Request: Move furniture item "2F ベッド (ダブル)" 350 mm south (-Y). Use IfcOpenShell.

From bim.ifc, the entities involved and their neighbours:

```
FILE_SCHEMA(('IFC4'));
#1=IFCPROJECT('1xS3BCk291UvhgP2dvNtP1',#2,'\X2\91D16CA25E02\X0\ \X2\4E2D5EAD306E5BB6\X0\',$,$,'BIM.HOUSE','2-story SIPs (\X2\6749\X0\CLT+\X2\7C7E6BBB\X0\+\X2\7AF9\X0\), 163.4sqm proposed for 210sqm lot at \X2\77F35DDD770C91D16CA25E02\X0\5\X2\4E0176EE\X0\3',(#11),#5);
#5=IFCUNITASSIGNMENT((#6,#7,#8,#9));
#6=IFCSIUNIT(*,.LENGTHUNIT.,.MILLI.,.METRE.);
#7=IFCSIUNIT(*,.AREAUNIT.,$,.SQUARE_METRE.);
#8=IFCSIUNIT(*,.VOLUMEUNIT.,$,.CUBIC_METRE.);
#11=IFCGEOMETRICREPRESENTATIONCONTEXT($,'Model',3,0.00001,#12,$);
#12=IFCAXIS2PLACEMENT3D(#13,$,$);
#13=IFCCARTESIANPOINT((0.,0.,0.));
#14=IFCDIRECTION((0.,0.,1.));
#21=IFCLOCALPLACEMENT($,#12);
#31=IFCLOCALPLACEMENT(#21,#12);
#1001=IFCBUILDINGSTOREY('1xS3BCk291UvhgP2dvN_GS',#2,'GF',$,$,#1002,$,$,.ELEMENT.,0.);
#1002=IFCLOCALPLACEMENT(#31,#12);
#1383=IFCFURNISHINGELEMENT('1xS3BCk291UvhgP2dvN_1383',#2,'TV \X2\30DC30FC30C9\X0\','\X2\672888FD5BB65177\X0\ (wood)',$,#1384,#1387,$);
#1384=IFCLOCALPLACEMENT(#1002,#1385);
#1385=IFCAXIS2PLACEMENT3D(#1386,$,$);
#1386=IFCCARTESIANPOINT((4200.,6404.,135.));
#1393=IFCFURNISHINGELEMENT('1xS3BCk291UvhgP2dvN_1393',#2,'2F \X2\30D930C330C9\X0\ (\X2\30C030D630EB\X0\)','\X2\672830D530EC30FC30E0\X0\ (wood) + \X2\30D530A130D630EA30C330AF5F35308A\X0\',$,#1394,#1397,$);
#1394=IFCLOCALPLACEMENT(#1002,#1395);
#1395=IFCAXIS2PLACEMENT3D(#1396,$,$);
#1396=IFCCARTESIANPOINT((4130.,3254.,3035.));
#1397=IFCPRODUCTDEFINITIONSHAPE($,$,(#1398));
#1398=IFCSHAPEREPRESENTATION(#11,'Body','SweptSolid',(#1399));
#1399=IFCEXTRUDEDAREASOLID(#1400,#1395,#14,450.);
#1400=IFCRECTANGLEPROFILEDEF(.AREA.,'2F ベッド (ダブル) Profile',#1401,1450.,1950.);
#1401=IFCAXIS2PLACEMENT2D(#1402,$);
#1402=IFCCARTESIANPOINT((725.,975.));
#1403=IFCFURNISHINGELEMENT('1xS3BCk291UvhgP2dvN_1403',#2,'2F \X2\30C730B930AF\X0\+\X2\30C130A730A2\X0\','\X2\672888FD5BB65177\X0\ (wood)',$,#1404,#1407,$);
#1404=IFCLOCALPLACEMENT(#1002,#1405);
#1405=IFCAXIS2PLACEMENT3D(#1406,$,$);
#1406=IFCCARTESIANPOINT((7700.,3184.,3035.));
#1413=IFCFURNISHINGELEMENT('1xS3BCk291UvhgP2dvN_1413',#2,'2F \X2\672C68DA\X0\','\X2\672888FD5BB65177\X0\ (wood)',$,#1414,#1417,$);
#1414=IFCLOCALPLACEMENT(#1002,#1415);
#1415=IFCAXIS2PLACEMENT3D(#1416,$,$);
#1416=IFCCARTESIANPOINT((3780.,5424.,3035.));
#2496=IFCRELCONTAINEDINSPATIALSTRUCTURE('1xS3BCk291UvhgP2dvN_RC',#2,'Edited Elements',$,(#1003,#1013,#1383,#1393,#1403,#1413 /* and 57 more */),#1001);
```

```python
import ifcopenshell
import ifcopenshell.api.geometry
import ifcopenshell.util.placement
import ifcopenshell.util.unit

model = ifcopenshell.open("bim.ifc")
unit_scale = ifcopenshell.util.unit.calculate_unit_scale(model)

item = model.by_id(1393)
matrix = ifcopenshell.util.placement.get_local_placement(item.ObjectPlacement)
matrix[1, 3] -= 0.35 / unit_scale
ifcopenshell.api.geometry.edit_object_placement(model, product=item, matrix=matrix, is_si=False)

print(ifcopenshell.util.placement.get_local_placement(item.ObjectPlacement).round(3) + 0.0)

model.write("bim_v2.ifc")
```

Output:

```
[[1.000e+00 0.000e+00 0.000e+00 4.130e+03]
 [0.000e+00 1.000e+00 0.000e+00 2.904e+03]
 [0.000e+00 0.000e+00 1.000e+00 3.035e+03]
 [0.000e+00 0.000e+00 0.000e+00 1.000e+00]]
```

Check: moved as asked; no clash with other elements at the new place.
